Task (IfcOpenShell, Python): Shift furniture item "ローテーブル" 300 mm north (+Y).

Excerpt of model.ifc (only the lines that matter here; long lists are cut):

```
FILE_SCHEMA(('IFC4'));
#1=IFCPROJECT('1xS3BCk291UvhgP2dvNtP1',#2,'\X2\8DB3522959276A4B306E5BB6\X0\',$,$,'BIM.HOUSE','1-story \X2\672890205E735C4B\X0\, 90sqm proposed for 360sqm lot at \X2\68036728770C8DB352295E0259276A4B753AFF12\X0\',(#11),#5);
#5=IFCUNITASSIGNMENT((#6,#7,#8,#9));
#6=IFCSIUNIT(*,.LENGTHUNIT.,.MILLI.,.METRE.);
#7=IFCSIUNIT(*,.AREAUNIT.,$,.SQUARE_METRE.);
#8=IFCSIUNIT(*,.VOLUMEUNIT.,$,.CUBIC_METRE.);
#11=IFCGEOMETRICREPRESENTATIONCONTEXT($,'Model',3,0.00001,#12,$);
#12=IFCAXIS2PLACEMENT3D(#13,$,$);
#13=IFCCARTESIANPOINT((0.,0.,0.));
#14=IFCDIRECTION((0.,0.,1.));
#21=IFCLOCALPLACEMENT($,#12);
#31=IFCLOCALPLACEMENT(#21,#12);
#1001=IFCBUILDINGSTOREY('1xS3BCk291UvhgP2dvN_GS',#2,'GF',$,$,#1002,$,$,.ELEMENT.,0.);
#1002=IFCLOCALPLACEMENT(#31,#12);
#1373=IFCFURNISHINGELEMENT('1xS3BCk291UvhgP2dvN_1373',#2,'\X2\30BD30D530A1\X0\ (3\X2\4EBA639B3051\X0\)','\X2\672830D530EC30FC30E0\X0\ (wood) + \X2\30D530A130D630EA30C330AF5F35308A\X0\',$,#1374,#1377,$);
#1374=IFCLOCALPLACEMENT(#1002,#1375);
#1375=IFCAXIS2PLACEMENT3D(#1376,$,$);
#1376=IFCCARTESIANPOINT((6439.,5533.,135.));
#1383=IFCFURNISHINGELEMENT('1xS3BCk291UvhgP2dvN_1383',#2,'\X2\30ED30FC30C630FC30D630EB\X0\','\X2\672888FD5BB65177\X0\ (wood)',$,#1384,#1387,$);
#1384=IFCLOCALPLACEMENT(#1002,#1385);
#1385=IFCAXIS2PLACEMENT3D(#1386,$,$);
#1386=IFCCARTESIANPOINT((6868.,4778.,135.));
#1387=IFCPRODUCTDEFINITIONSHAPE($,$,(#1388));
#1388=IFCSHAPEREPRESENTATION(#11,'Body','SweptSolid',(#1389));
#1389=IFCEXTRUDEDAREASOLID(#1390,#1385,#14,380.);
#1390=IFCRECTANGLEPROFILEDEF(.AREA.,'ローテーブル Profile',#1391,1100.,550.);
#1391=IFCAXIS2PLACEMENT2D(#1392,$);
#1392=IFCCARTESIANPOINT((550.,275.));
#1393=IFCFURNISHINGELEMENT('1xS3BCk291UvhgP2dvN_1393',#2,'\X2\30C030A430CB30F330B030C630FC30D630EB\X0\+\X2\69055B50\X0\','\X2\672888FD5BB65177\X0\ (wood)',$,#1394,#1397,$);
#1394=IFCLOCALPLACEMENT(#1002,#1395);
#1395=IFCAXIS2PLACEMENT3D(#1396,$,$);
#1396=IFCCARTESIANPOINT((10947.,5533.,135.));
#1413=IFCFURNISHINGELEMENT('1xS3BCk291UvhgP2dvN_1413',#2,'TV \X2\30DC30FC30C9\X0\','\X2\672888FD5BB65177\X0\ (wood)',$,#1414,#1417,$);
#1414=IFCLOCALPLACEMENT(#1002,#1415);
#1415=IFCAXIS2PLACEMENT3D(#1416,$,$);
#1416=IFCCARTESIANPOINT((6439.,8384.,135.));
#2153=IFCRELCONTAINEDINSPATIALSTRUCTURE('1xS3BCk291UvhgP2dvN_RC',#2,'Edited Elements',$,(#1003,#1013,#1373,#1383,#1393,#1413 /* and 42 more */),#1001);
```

```python
import ifcopenshell
import ifcopenshell.api.geometry
import ifcopenshell.util.placement
import ifcopenshell.util.unit

model = ifcopenshell.open("model.ifc")
unit_scale = ifcopenshell.util.unit.calculate_unit_scale(model)

item = model.by_id(1383)
matrix = ifcopenshell.util.placement.get_local_placement(item.ObjectPlacement)
matrix[1, 3] += 0.3 / unit_scale
ifcopenshell.api.geometry.edit_object_placement(model, product=item, matrix=matrix, is_si=False)

print(ifcopenshell.util.placement.get_local_placement(item.ObjectPlacement).round(3) + 0.0)

model.write("model_updated.ifc")
```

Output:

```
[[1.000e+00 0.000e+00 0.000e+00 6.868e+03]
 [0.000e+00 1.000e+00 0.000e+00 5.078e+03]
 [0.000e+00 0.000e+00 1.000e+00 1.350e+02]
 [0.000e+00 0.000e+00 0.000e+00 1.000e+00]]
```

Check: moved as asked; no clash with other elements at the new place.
